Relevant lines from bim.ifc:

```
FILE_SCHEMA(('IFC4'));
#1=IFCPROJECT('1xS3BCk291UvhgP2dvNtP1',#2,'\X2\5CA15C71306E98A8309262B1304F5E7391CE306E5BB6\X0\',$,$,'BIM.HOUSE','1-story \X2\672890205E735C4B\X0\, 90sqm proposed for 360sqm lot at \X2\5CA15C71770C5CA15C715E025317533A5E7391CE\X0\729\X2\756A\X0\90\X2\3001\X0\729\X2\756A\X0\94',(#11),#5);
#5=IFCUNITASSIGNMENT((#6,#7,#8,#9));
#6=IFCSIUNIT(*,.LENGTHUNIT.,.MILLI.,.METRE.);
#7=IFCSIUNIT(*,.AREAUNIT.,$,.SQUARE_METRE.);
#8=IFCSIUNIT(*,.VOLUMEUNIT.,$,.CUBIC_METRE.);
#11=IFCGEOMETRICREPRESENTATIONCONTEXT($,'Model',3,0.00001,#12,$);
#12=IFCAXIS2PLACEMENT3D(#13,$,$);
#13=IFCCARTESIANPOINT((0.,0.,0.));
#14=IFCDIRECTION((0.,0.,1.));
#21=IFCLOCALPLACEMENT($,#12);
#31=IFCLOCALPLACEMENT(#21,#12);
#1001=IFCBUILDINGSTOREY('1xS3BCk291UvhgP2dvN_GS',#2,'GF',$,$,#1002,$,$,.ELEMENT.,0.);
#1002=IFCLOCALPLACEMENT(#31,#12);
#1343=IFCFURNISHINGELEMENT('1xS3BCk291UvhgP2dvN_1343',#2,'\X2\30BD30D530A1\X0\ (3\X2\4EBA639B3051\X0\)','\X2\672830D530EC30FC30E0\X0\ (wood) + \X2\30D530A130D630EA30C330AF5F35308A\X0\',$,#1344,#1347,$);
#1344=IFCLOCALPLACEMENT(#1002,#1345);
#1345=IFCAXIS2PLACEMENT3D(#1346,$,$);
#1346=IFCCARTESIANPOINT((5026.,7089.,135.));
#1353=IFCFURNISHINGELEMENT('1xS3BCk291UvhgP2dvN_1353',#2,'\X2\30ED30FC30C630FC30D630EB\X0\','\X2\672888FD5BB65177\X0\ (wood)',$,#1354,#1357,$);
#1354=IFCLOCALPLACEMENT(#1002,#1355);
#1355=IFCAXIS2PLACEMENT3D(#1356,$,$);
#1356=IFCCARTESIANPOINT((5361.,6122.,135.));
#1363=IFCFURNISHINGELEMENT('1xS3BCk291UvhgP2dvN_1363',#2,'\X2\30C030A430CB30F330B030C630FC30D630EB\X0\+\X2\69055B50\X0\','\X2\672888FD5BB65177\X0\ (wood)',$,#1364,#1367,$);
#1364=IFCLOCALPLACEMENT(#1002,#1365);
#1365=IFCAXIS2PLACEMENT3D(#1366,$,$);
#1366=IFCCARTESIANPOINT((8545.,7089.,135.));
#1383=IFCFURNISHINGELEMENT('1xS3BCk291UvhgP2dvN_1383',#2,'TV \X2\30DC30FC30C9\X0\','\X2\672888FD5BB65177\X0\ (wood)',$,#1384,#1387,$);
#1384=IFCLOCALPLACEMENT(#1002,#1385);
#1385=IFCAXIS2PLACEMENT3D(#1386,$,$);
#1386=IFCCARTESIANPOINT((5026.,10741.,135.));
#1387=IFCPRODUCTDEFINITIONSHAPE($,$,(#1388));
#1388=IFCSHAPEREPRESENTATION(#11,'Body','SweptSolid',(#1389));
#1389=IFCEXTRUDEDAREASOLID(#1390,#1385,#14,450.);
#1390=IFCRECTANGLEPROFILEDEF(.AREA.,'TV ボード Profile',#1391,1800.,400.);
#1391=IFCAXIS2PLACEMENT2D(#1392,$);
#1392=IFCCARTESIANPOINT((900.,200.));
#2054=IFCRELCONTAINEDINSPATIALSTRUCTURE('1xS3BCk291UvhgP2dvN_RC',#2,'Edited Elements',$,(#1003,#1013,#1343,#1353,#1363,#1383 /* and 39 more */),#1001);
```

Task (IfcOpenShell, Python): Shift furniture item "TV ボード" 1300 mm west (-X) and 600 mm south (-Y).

```python
import ifcopenshell
import ifcopenshell.api.geometry
import ifcopenshell.util.placement
import ifcopenshell.util.unit

model = ifcopenshell.open("bim.ifc")
unit_scale = ifcopenshell.util.unit.calculate_unit_scale(model)

item = model.by_id(1383)
matrix = ifcopenshell.util.placement.get_local_placement(item.ObjectPlacement)
matrix[0, 3] -= 1.3 / unit_scale
matrix[1, 3] -= 0.6 / unit_scale
ifcopenshell.api.geometry.edit_object_placement(model, product=item, matrix=matrix, is_si=False)

print(ifcopenshell.util.placement.get_local_placement(item.ObjectPlacement).round(3) + 0.0)

model.write("bim_updated.ifc")
```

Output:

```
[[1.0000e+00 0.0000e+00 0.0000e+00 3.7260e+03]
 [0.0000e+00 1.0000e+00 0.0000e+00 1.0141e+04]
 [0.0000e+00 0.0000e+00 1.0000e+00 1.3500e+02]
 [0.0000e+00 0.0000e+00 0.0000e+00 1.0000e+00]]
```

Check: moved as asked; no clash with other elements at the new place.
